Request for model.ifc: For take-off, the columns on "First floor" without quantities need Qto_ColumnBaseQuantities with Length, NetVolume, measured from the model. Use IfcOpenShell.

First a look at what the model holds.

```python
import ifcopenshell
import ifcopenshell.util.element
import ifcopenshell.util.unit

model = ifcopenshell.open("model.ifc")
print(model.schema)
for unit_type in ("LENGTHUNIT", "AREAUNIT", "VOLUMEUNIT"):
    print(unit_type, ifcopenshell.util.unit.calculate_unit_scale(model, unit_type))
storey = next(s for s in model.by_type("IfcBuildingStorey") if s.Name == "First floor")
columns = [e for e in ifcopenshell.util.element.get_decomposition(storey) if e.is_a("IfcColumn")]
for e in sorted(columns, key=lambda e: e.id()):
    print(e.id(), e.is_a(), e.Name, list(ifcopenshell.util.element.get_psets(e, qtos_only=True)), sep=" | ")
```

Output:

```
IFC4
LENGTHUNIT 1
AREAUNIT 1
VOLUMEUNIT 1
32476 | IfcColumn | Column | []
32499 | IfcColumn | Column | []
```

```python
import ifcopenshell
import ifcopenshell.api.pset
import ifcopenshell.geom
import ifcopenshell.util.element
import ifcopenshell.util.shape
import ifcopenshell.util.unit

model = ifcopenshell.open("model.ifc")
unit_scale = ifcopenshell.util.unit.calculate_unit_scale(model)
volume_scale = ifcopenshell.util.unit.calculate_unit_scale(model, "VOLUMEUNIT")
settings = ifcopenshell.geom.settings()

storey = next(s for s in model.by_type("IfcBuildingStorey") if s.Name == "First floor")
columns = [e for e in ifcopenshell.util.element.get_decomposition(storey) if e.is_a("IfcColumn")]

for e in sorted(columns, key=lambda e: e.id()):
    if ifcopenshell.util.element.get_psets(e, qtos_only=True, should_inherit=False):
        continue
    # Geometry comes back in metres, in the element's own axes.
    shape = ifcopenshell.geom.create_shape(settings, e)
    values = {
        "Length": ifcopenshell.util.shape.get_z(shape.geometry) / unit_scale,
        "NetVolume": ifcopenshell.util.shape.get_volume(shape.geometry) / volume_scale,
    }
    qto = ifcopenshell.api.pset.add_qto(model, product=e, name="Qto_ColumnBaseQuantities")
    ifcopenshell.api.pset.edit_qto(model, qto=qto, properties=values)
    print(e.id(), {k: round(v, 3) for k, v in values.items()})

model.write("model_updated.ifc")
```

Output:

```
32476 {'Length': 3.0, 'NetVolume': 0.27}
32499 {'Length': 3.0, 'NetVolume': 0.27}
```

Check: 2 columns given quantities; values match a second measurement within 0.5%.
